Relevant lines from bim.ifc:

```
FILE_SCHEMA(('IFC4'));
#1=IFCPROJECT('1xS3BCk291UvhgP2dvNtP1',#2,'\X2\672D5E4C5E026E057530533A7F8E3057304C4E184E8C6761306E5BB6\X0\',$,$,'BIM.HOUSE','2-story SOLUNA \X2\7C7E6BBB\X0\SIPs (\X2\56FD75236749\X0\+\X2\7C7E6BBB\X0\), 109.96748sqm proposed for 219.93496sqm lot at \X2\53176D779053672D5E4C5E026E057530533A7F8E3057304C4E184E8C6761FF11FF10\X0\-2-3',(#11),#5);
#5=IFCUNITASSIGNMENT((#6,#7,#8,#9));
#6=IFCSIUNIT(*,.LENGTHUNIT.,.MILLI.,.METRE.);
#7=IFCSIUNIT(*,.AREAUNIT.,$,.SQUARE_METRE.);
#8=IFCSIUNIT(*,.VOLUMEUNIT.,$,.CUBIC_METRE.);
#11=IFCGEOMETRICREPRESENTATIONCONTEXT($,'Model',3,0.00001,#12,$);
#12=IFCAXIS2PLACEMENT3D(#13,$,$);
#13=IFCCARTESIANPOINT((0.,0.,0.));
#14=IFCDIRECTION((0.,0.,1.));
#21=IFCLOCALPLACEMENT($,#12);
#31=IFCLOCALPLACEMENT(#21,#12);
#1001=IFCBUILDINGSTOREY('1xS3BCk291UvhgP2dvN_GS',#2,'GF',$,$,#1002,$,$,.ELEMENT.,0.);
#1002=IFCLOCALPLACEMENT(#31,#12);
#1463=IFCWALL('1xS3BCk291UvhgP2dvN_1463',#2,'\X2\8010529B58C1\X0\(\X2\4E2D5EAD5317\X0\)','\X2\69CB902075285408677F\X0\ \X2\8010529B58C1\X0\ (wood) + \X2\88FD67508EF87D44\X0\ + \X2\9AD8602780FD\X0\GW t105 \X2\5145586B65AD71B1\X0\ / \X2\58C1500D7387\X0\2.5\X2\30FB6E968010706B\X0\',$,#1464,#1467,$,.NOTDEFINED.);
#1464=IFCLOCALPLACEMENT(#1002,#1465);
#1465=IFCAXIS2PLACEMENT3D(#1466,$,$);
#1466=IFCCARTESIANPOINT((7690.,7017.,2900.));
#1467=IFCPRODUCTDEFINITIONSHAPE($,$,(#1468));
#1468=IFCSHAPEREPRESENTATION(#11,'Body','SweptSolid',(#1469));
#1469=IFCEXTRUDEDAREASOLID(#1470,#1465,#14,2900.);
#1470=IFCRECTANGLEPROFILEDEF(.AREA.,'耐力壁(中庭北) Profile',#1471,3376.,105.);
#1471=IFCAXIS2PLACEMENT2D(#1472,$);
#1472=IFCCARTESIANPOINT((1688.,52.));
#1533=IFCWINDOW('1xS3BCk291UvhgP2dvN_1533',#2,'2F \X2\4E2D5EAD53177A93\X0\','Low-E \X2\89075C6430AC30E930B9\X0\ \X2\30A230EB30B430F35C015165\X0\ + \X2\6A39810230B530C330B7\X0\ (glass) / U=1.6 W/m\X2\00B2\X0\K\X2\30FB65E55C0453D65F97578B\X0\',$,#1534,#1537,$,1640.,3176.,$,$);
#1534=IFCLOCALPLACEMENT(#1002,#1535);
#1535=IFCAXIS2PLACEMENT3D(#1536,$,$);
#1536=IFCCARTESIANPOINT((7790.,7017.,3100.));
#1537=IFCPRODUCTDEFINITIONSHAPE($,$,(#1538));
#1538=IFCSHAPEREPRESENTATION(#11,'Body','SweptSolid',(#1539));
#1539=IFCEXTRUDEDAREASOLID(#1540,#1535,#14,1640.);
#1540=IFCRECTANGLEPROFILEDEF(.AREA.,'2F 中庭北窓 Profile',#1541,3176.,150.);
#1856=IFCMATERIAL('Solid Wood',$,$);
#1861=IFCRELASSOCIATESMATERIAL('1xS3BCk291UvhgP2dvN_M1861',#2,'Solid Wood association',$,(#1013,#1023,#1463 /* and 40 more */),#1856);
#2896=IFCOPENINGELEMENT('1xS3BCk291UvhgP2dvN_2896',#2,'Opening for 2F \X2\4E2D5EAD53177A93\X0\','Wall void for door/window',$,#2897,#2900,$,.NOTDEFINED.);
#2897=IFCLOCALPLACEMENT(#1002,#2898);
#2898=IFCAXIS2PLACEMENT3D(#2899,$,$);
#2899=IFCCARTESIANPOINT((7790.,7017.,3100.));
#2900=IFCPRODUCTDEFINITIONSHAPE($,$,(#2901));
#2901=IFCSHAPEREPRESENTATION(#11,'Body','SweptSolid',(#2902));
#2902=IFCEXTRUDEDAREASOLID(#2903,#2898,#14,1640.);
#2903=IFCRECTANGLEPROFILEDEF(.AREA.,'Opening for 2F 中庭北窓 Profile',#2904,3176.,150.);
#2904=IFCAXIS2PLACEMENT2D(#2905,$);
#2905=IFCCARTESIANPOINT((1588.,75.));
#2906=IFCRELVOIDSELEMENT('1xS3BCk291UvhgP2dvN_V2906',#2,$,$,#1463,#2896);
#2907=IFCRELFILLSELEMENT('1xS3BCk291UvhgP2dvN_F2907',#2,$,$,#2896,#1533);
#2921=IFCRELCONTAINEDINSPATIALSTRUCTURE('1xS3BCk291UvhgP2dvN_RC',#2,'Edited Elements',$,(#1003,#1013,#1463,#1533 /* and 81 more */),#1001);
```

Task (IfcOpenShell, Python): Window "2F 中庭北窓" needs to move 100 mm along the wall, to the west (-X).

```python
import ifcopenshell
import ifcopenshell.api.geometry
import ifcopenshell.util.placement

model = ifcopenshell.open("bim.ifc")

window = model.by_guid("1xS3BCk291UvhgP2dvN_1533")
opening = window.FillsVoids[0].RelatingOpeningElement
wall = opening.VoidsElements[0].RelatingBuildingElement

wall_matrix = ifcopenshell.util.placement.get_local_placement(wall.ObjectPlacement)
shift = wall_matrix[:3, 0] * -100.0
before = ifcopenshell.util.placement.get_local_placement(window.ObjectPlacement)[:3, 3].copy()

# The window is not placed relative to its opening, so move both.
for product in (opening, window):
    matrix = ifcopenshell.util.placement.get_local_placement(product.ObjectPlacement)
    matrix[:3, 3] += shift
    ifcopenshell.api.geometry.edit_object_placement(model, product=product, matrix=matrix, is_si=False)

after = ifcopenshell.util.placement.get_local_placement(window.ObjectPlacement)[:3, 3]
print("window moved by", (after - before).round(3) + 0.0)

model.write("bim-out.ifc")
```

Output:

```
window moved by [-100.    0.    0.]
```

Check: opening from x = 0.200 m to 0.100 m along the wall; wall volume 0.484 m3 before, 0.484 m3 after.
